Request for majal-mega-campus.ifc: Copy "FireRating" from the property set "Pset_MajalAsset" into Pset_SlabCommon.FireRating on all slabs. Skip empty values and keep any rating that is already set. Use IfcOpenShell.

First a look at what the model holds.

```python
import ifcopenshell
import ifcopenshell.util.element

model = ifcopenshell.open("majal-mega-campus.ifc")
print(model.schema)
slabs = model.by_type("IfcSlab")
print(len(slabs), "slabs")
for e in slabs[:8]:
    source = ifcopenshell.util.element.get_pset(e, "Pset_MajalAsset", "FireRating")
    target = ifcopenshell.util.element.get_pset(e, "Pset_SlabCommon", "FireRating")
    print(e.id(), repr(source), repr(target), sep=" | ")
```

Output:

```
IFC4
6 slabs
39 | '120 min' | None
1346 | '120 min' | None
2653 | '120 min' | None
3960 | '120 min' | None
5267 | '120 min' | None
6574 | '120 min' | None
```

```python
import ifcopenshell
import ifcopenshell.api.pset
import ifcopenshell.util.element

model = ifcopenshell.open("majal-mega-campus.ifc")

count = 0
for e in model.by_type("IfcSlab"):
    value = ifcopenshell.util.element.get_pset(e, "Pset_MajalAsset", "FireRating")
    current = ifcopenshell.util.element.get_pset(e, "Pset_SlabCommon", "FireRating")
    if not value or not value.strip() or current:
        continue
    # add_pset returns the element's existing set when there is one.
    pset = ifcopenshell.api.pset.add_pset(model, product=e, name="Pset_SlabCommon")
    ifcopenshell.api.pset.edit_pset(model, pset=pset, properties={"FireRating": value})
    count += 1

print(count, "slabs updated")

model.write("majal-mega-campus_edited.ifc")
```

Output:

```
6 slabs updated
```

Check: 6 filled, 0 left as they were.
